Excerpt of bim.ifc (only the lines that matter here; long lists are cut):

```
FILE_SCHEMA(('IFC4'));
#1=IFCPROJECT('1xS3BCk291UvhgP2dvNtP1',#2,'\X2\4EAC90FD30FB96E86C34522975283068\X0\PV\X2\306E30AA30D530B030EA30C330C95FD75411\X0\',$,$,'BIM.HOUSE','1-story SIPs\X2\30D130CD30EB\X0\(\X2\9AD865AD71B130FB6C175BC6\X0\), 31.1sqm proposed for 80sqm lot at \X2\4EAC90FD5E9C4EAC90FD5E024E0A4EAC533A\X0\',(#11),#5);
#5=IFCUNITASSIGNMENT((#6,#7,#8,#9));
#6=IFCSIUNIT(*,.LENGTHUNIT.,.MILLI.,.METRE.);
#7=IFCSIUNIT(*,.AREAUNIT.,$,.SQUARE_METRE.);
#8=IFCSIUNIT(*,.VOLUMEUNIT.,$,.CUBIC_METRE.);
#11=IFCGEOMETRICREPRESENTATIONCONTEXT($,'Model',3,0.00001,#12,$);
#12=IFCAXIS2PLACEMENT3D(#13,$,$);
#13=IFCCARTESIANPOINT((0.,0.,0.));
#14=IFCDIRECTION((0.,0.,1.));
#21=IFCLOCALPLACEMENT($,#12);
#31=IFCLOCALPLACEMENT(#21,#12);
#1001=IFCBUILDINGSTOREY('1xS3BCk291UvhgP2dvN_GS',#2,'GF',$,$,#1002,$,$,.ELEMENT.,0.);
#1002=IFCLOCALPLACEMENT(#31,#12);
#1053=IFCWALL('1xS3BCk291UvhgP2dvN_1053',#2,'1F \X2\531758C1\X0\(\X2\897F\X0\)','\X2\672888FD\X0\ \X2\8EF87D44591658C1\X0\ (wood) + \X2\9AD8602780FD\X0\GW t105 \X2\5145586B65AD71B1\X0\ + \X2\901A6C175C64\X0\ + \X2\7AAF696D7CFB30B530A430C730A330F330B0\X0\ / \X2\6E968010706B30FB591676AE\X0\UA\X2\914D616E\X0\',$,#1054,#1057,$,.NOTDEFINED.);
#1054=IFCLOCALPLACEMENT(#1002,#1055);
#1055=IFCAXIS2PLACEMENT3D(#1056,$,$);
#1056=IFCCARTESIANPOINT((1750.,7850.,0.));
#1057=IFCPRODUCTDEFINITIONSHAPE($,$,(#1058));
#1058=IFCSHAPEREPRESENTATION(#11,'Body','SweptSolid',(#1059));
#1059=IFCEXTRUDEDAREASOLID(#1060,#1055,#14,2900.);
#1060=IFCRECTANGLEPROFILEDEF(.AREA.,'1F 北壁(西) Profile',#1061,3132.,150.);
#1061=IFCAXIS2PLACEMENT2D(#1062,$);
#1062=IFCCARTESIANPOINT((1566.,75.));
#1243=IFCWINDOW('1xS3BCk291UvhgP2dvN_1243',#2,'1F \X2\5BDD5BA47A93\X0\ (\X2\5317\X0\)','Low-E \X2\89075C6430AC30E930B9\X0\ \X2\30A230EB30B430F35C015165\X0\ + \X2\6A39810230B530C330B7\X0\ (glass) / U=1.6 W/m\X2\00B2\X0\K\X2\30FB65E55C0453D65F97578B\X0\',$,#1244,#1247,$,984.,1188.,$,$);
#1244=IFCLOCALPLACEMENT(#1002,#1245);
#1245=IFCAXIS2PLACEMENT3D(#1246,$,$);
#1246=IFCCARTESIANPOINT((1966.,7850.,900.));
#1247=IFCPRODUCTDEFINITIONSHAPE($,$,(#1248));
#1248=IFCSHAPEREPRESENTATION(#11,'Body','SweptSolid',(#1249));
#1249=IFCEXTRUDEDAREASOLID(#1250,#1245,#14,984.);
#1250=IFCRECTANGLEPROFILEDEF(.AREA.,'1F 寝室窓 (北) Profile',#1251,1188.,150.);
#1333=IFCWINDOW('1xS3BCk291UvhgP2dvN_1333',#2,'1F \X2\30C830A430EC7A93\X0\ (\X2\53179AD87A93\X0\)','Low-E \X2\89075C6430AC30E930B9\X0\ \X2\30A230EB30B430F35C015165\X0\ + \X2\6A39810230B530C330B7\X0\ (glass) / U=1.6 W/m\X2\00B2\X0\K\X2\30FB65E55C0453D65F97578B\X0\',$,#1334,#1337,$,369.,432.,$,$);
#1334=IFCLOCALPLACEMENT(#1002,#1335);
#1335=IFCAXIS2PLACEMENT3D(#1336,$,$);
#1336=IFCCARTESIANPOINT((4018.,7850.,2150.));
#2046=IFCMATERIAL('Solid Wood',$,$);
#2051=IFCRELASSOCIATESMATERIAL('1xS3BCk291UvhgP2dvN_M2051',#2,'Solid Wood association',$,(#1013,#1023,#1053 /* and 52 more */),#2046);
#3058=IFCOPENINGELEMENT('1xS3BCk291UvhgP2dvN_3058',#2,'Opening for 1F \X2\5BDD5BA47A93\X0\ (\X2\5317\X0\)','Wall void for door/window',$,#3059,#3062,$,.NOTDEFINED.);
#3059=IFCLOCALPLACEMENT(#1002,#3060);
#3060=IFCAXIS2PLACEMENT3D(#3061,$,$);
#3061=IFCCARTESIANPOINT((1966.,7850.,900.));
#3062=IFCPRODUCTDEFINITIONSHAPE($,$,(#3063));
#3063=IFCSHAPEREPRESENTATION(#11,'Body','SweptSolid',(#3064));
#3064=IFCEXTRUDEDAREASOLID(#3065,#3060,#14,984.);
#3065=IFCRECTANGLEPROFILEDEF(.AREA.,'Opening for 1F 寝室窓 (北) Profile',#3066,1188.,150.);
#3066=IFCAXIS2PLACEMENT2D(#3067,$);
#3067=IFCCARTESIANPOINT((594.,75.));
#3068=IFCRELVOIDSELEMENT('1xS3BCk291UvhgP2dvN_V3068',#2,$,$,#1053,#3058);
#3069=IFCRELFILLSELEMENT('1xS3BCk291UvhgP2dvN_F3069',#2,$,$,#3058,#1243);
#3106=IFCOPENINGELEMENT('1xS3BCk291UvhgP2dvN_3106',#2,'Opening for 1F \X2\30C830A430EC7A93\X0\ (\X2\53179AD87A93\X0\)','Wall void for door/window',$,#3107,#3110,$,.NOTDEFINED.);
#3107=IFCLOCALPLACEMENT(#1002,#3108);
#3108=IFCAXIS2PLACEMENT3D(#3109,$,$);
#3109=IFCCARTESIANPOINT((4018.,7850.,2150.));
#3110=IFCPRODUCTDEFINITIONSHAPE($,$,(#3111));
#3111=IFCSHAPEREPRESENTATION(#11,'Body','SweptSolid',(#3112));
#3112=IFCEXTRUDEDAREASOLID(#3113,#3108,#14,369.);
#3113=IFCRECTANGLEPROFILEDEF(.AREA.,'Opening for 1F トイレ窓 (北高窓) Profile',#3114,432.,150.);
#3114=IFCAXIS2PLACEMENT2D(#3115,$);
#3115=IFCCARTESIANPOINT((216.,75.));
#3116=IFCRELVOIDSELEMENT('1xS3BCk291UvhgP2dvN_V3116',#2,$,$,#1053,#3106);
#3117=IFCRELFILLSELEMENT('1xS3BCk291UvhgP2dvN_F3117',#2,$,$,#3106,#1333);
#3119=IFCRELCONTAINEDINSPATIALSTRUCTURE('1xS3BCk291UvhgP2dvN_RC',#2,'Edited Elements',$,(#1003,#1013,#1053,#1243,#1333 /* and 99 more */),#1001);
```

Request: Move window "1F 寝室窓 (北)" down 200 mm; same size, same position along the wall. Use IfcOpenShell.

```python
import numpy as np
import ifcopenshell
import ifcopenshell.api.geometry
import ifcopenshell.util.placement
import ifcopenshell.util.unit

model = ifcopenshell.open("bim.ifc")
unit_scale = ifcopenshell.util.unit.calculate_unit_scale(model)

window = model.by_guid("1xS3BCk291UvhgP2dvN_1243")
opening = window.FillsVoids[0].RelatingOpeningElement
dz = -0.2 / unit_scale

shift = np.array([0.0, 0.0, dz])
# The window is not placed relative to its opening, so move both.
for product in (opening, window):
    matrix = ifcopenshell.util.placement.get_local_placement(product.ObjectPlacement)
    matrix[:3, 3] += shift
    ifcopenshell.api.geometry.edit_object_placement(model, product=product, matrix=matrix, is_si=False)

print(f"moved by {dz * unit_scale:+.3f} m")

model.write("bim_updated.ifc")
```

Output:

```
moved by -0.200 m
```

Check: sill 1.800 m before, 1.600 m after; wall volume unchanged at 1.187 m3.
